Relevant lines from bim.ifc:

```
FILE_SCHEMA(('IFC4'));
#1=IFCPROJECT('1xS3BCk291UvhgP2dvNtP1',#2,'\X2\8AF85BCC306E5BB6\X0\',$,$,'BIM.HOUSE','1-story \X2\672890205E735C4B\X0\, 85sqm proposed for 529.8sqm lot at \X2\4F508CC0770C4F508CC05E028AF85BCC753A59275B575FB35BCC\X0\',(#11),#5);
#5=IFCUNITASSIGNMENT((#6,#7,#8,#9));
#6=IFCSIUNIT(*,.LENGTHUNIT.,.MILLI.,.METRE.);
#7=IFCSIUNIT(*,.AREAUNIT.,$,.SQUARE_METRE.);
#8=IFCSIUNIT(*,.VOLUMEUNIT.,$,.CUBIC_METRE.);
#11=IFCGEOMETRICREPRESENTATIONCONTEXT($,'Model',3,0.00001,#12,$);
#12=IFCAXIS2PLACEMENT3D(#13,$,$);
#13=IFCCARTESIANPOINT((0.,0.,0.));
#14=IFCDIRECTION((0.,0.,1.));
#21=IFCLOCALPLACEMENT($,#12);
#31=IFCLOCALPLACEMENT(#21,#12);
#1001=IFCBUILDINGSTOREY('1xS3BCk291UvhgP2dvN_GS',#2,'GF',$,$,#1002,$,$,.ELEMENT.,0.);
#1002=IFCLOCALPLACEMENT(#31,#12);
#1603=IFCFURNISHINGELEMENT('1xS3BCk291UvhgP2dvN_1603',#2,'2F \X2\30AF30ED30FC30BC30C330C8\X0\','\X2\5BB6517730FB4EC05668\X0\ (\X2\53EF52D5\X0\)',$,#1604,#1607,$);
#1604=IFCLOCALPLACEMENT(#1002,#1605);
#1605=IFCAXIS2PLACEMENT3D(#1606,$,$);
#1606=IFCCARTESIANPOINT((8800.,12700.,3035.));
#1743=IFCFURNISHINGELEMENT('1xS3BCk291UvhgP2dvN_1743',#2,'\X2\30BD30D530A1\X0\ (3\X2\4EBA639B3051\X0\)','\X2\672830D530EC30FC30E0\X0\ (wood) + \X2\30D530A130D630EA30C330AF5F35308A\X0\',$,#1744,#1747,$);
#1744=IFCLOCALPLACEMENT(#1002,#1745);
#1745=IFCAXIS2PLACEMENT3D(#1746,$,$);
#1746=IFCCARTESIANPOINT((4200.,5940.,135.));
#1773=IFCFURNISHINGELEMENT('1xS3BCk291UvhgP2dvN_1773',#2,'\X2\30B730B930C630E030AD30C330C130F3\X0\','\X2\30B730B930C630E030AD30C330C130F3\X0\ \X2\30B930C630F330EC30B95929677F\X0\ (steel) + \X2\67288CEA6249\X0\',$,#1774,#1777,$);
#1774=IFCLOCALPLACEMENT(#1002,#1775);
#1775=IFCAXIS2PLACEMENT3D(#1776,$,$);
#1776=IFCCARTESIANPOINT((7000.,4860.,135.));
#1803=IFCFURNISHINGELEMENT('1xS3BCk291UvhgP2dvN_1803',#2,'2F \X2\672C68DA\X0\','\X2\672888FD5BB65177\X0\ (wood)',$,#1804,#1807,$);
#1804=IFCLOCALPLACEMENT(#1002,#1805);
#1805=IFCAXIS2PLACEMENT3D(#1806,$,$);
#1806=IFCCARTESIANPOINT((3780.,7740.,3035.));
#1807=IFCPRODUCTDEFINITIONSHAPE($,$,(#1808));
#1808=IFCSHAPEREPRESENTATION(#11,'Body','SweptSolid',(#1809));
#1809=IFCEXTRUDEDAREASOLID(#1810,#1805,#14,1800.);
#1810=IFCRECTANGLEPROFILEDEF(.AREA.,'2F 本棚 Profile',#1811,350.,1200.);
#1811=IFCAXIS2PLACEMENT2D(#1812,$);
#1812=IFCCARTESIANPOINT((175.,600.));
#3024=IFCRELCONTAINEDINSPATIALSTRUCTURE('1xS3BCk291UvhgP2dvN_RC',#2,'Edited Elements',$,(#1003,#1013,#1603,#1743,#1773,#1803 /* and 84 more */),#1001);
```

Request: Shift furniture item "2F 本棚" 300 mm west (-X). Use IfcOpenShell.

```python
import ifcopenshell
import ifcopenshell.api.geometry
import ifcopenshell.util.placement

model = ifcopenshell.open("bim.ifc")

item = model.by_guid("1xS3BCk291UvhgP2dvN_1803")
matrix = ifcopenshell.util.placement.get_local_placement(item.ObjectPlacement)
matrix[0, 3] -= 300.0
ifcopenshell.api.geometry.edit_object_placement(model, product=item, matrix=matrix, is_si=False)

print(ifcopenshell.util.placement.get_local_placement(item.ObjectPlacement).round(3) + 0.0)

model.write("bim_rev.ifc")
```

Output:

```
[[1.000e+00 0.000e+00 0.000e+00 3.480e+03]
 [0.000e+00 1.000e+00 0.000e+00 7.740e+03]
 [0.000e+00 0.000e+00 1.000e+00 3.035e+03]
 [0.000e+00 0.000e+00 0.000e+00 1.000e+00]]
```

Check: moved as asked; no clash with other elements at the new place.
